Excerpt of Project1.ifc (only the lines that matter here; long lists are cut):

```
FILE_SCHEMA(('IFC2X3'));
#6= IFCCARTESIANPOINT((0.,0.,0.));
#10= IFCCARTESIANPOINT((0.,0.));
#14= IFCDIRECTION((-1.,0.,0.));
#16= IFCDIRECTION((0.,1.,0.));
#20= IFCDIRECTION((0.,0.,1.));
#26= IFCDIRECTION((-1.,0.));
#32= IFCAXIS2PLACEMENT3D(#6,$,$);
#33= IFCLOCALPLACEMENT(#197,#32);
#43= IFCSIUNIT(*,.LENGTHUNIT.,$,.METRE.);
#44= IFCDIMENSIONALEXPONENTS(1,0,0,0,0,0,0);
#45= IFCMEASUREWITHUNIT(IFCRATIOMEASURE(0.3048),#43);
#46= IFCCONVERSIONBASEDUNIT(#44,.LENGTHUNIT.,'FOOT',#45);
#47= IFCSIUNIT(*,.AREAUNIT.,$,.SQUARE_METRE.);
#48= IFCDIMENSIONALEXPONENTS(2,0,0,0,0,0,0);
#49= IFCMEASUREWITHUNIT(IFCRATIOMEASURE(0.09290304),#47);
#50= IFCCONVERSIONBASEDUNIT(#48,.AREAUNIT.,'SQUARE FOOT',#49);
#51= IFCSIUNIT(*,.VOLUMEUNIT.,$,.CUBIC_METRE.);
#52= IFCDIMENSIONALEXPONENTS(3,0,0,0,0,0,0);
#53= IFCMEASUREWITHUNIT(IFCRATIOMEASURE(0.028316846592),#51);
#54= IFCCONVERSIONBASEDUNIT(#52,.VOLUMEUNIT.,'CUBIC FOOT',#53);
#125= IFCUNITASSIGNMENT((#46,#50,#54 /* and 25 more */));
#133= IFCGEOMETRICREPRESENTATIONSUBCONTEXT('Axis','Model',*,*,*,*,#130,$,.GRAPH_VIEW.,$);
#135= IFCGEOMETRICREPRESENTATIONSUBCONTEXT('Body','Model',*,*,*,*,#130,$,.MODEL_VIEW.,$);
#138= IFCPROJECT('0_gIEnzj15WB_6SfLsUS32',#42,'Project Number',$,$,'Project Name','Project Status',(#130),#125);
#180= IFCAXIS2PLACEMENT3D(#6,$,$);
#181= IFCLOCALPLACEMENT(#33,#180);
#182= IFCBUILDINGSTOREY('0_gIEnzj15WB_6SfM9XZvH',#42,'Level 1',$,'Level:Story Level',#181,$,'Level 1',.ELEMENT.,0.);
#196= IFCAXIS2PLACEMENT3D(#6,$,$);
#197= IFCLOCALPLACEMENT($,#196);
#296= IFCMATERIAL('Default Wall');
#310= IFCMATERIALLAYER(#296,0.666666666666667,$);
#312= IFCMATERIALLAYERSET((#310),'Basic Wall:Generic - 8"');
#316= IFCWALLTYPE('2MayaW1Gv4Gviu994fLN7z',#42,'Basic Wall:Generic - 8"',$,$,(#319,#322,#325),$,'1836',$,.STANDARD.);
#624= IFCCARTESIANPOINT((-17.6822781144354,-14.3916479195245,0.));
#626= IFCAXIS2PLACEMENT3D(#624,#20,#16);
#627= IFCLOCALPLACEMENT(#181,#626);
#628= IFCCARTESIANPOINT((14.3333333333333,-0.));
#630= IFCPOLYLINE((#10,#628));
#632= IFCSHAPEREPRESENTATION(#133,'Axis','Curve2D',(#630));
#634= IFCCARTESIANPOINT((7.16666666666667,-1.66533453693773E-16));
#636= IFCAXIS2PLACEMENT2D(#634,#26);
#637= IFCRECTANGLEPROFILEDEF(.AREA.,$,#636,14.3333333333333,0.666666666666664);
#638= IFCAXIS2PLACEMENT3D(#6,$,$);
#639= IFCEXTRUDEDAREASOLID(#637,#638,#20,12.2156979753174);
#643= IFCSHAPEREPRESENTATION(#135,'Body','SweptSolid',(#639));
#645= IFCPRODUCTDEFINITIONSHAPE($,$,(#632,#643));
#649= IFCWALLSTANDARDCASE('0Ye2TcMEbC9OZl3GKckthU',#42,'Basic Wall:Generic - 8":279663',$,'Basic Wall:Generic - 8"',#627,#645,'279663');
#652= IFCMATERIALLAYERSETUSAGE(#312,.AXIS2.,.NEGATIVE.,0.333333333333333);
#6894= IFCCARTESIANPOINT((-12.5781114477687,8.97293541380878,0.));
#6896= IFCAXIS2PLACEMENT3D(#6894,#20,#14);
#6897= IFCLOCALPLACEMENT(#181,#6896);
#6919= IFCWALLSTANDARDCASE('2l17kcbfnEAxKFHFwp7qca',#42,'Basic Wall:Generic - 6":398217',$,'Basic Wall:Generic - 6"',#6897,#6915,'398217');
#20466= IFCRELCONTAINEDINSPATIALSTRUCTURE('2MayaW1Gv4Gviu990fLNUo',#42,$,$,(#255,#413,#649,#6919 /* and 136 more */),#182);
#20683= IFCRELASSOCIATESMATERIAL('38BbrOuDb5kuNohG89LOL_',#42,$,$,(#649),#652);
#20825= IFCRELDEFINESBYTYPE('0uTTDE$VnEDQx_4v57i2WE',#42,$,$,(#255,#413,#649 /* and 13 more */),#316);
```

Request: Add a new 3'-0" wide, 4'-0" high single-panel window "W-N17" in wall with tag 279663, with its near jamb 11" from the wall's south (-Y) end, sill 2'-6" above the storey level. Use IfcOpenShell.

```python
import numpy as np
import ifcopenshell
import ifcopenshell.api.feature
import ifcopenshell.api.geometry
import ifcopenshell.api.root
import ifcopenshell.api.spatial
import ifcopenshell.api.type
import ifcopenshell.geom
import ifcopenshell.util.element
import ifcopenshell.util.placement
import ifcopenshell.util.representation
import ifcopenshell.util.shape
import ifcopenshell.util.unit

model = ifcopenshell.open("Project1.ifc")
unit_scale = ifcopenshell.util.unit.calculate_unit_scale(model)
settings = ifcopenshell.geom.settings()


def volume(element):
    """Net volume in cubic metres, openings subtracted."""
    shape = ifcopenshell.geom.create_shape(settings, element)
    return ifcopenshell.util.shape.get_volume(shape.geometry)


wall = model.by_id(649)
storey = ifcopenshell.util.element.get_container(wall, ifc_class="IfcBuildingStorey")
context = ifcopenshell.util.representation.get_context(model, "Model", "Body", "MODEL_VIEW")
before = volume(wall)

width, height, from_end, sill = 0.9144, 1.2192, 0.2794, 0.762  # metres

# The wall runs along its own X axis, and the end named is its -X end.
wall_shape = ifcopenshell.geom.create_shape(settings, wall)
x, y, z = ifcopenshell.util.shape.get_vertices(wall_shape.geometry).T
start = x.min() + from_end
face, thickness = float(y.min()), float(y.max() - y.min())
wall_matrix = ifcopenshell.util.placement.get_local_placement(wall.ObjectPlacement)
level = ifcopenshell.util.placement.get_local_placement(storey.ObjectPlacement)[2, 3]


def in_wall(x, y):
    """Placement at x, y metres in the wall's axes, at sill height."""
    matrix = wall_matrix.copy()
    matrix[:, 3] = wall_matrix @ np.array([x / unit_scale, y / unit_scale, 0.0, 1.0])
    matrix[2, 3] = level + sill / unit_scale
    return matrix


# Opening: a box that overshoots both wall faces by 50 mm.
opening = ifcopenshell.api.root.create_entity(model, ifc_class="IfcOpeningElement")
box = ifcopenshell.api.geometry.add_wall_representation(
    model, context=context, length=width, height=height, thickness=thickness + 0.1
)
ifcopenshell.api.geometry.assign_representation(model, product=opening, representation=box)
ifcopenshell.api.geometry.edit_object_placement(model, product=opening, matrix=in_wall(start, face - 0.05), is_si=False)
ifcopenshell.api.feature.add_feature(model, feature=opening, element=wall)

window = ifcopenshell.api.root.create_entity(model, ifc_class="IfcWindow", name="W-N17")
window.OverallWidth, window.OverallHeight = width / unit_scale, height / unit_scale
body = ifcopenshell.api.geometry.add_window_representation(
    model,
    context=context,
    overall_width=window.OverallWidth,
    overall_height=window.OverallHeight,
    partition_type="SINGLE_PANEL",
)
ifcopenshell.api.geometry.assign_representation(model, product=window, representation=body)
ifcopenshell.api.spatial.assign_container(model, products=[window], relating_structure=storey)
fills = ifcopenshell.api.feature.add_filling(model, opening=opening, element=window)
fills.OwnerHistory = window.OwnerHistory  # required in IFC2X3

# IFC2X3 keeps the operation on the window style.
style = ifcopenshell.api.root.create_entity(model, ifc_class="IfcWindowStyle", name="W-N17")
style.OperationType, style.ConstructionType = "SINGLE_PANEL", "NOTDEFINED"
style.ParameterTakesPrecedence = style.Sizeable = False
ifcopenshell.api.type.assign_type(model, related_objects=[window], relating_type=style)

# Centre the window in the wall's thickness.
ifcopenshell.api.geometry.edit_object_placement(model, product=window, matrix=in_wall(start, face), is_si=False)
window_shape = ifcopenshell.geom.create_shape(settings, window)
depth = ifcopenshell.util.shape.get_vertices(window_shape.geometry)[:, 1]
offset = face + thickness / 2 - (depth.min() + depth.max()) / 2
ifcopenshell.api.geometry.edit_object_placement(model, product=window, matrix=in_wall(start, offset), is_si=False)

after = volume(wall)

print(f"wall volume {before:.3f} -> {after:.3f} m3")

model.write("Project1-out.ifc")
```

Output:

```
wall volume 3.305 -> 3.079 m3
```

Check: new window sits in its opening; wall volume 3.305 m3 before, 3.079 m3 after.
